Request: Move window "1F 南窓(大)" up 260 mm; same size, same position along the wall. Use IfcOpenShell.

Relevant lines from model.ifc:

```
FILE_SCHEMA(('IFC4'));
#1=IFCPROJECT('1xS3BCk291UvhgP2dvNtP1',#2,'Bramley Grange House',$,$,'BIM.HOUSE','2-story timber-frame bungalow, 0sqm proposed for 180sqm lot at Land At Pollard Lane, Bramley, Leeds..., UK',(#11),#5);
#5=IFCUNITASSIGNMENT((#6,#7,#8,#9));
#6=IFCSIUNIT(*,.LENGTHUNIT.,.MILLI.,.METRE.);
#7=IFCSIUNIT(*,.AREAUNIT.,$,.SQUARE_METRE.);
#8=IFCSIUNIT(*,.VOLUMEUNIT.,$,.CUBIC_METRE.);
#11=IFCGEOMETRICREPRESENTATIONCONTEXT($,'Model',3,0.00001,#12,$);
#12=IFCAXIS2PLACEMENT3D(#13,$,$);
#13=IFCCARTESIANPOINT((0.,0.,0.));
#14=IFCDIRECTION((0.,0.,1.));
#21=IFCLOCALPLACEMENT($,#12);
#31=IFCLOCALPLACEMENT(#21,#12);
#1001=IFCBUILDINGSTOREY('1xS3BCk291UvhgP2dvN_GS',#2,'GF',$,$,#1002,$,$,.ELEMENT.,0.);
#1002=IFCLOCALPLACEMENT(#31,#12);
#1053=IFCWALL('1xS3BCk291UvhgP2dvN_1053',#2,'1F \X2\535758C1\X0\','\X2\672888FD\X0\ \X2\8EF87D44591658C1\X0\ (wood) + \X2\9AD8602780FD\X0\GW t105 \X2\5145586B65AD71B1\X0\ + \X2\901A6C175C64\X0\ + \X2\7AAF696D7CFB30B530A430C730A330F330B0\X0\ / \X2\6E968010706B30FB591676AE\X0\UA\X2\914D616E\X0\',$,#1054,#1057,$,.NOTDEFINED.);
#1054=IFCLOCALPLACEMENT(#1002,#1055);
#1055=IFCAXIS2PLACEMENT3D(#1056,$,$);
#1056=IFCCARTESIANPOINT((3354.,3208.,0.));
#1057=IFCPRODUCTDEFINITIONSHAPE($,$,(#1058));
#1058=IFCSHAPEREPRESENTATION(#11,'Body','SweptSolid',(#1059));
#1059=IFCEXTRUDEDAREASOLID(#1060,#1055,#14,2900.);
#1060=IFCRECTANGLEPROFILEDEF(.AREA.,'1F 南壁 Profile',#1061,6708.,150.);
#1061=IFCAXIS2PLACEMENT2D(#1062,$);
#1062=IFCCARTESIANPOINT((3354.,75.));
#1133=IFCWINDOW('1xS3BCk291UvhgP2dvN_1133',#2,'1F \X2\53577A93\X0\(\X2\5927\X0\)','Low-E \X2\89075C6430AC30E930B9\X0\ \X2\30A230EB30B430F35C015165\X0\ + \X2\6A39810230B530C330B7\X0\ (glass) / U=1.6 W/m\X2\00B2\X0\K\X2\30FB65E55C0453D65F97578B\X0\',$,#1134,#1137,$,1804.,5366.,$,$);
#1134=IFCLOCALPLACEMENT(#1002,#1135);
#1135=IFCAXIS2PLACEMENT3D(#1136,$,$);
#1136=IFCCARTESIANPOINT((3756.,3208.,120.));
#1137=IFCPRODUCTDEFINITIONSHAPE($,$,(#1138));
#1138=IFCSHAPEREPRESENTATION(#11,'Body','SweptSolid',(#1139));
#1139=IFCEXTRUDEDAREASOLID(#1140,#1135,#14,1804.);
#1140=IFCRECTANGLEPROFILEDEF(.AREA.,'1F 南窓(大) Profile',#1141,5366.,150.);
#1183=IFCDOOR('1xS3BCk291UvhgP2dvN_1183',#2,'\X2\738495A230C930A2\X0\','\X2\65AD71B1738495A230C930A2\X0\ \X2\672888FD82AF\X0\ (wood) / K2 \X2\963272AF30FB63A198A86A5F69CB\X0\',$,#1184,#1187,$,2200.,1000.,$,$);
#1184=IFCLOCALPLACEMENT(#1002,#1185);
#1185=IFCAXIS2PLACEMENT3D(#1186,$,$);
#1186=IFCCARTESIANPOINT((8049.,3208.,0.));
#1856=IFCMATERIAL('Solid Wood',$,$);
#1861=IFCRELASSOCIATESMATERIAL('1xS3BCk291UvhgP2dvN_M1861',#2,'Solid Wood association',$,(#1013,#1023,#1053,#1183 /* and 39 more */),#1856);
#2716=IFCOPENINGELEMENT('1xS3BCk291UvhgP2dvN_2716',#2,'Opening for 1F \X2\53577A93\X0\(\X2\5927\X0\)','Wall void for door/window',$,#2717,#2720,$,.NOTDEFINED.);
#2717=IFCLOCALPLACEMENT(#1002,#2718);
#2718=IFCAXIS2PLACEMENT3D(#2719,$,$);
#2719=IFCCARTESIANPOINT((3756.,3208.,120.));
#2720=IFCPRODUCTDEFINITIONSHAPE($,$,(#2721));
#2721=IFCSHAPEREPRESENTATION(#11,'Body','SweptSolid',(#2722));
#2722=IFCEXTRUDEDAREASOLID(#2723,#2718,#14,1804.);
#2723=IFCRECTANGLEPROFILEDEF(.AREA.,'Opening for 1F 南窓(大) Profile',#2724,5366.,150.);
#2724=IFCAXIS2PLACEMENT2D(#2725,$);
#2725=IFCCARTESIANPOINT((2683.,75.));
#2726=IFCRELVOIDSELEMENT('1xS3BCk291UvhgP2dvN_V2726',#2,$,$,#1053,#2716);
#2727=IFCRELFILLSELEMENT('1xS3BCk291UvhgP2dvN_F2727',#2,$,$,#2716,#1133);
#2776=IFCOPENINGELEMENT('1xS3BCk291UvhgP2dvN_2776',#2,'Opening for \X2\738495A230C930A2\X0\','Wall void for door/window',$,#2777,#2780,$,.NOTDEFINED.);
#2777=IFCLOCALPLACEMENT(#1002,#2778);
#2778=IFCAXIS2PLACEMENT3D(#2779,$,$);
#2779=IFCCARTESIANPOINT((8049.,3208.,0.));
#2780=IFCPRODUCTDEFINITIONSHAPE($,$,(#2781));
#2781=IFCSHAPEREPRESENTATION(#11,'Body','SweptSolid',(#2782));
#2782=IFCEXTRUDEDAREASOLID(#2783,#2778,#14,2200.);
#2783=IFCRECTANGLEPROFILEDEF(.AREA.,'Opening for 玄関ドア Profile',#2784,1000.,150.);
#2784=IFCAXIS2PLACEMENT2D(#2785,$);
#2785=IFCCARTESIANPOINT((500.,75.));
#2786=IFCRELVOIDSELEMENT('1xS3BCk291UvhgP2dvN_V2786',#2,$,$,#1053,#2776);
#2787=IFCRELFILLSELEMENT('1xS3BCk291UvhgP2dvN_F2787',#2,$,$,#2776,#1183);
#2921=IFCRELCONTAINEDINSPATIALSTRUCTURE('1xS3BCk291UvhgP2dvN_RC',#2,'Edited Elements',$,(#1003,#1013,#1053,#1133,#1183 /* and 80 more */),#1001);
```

```python
import numpy as np
import ifcopenshell
import ifcopenshell.api.geometry
import ifcopenshell.util.placement
import ifcopenshell.util.unit

model = ifcopenshell.open("model.ifc")
unit_scale = ifcopenshell.util.unit.calculate_unit_scale(model)

window = model.by_guid("1xS3BCk291UvhgP2dvN_1133")
opening = window.FillsVoids[0].RelatingOpeningElement
dz = 0.26 / unit_scale

shift = np.array([0.0, 0.0, dz])
# The window is not placed relative to its opening, so move both.
for product in (opening, window):
    matrix = ifcopenshell.util.placement.get_local_placement(product.ObjectPlacement)
    matrix[:3, 3] += shift
    ifcopenshell.api.geometry.edit_object_placement(model, product=product, matrix=matrix, is_si=False)

print(f"moved by {dz * unit_scale:+.3f} m")

model.write("model_v2.ifc")
```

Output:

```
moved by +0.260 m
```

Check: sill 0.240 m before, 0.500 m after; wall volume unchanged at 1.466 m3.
